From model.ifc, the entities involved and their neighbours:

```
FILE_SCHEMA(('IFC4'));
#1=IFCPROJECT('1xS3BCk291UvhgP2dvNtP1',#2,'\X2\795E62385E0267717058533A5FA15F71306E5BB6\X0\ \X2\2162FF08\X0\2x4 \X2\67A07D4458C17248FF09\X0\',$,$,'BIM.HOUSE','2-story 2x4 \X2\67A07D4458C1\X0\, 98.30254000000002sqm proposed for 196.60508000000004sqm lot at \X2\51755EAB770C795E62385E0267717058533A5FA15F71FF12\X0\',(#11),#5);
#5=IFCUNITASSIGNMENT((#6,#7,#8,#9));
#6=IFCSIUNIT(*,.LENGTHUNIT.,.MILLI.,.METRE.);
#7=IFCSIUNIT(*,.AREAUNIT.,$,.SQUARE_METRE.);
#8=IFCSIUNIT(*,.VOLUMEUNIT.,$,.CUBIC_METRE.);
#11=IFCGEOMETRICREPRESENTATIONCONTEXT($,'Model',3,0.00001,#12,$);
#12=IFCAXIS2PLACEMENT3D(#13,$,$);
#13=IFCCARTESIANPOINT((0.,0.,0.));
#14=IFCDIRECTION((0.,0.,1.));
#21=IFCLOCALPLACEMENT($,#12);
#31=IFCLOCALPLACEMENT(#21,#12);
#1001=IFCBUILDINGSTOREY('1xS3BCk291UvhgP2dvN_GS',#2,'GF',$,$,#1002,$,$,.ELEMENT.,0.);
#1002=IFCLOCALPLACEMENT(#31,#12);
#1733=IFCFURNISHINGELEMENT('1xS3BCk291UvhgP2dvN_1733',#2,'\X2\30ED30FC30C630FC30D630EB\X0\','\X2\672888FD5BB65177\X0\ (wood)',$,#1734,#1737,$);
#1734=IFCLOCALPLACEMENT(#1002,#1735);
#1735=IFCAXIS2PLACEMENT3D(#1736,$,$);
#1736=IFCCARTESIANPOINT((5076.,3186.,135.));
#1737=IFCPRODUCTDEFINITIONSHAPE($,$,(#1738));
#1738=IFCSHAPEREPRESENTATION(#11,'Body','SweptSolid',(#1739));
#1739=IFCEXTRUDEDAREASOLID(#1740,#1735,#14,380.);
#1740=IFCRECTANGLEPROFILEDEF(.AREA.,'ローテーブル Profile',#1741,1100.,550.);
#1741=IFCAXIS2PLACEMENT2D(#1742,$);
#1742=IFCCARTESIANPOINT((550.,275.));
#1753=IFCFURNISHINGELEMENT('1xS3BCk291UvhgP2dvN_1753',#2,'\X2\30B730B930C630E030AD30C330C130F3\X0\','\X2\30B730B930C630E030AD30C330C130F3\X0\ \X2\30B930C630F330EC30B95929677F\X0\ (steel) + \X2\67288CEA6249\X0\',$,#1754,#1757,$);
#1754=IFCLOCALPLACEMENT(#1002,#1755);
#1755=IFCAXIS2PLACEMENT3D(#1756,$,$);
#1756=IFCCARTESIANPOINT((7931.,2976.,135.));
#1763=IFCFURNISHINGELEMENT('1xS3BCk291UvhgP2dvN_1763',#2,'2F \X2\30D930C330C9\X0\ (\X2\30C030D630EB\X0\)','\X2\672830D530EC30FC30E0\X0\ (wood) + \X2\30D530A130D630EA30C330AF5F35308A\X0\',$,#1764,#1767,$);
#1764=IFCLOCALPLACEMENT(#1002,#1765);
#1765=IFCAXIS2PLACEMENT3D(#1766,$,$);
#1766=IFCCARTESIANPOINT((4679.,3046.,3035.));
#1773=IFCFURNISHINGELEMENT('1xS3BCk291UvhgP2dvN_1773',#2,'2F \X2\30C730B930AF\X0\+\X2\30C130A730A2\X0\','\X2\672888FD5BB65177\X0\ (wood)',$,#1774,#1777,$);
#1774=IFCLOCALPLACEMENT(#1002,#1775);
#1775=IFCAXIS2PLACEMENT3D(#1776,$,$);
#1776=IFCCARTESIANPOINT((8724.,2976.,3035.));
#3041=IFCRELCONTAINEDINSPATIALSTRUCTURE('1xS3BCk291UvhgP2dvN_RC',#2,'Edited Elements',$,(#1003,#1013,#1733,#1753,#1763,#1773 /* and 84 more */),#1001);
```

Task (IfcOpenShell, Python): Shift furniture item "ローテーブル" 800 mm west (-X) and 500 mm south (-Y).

```python
import ifcopenshell
import ifcopenshell.api.geometry
import ifcopenshell.util.placement
import ifcopenshell.util.unit

model = ifcopenshell.open("model.ifc")
unit_scale = ifcopenshell.util.unit.calculate_unit_scale(model)

item = model.by_guid("1xS3BCk291UvhgP2dvN_1733")
matrix = ifcopenshell.util.placement.get_local_placement(item.ObjectPlacement)
matrix[0, 3] -= 0.8 / unit_scale
matrix[1, 3] -= 0.5 / unit_scale
ifcopenshell.api.geometry.edit_object_placement(model, product=item, matrix=matrix, is_si=False)

print(ifcopenshell.util.placement.get_local_placement(item.ObjectPlacement).round(3) + 0.0)

model.write("model_edited.ifc")
```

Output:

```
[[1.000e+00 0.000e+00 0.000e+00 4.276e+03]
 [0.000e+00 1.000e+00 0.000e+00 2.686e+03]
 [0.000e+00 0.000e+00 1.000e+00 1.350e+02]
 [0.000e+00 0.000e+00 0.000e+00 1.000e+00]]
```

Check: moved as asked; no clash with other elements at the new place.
